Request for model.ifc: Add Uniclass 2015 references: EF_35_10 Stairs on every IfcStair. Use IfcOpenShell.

First a look at what the model holds.

```python
import ifcopenshell

model = ifcopenshell.open("model.ifc")
print(model.schema)
print("classifications:", [c.Name for c in model.by_type("IfcClassification")])
for ifc_class in ("IfcDoor", "IfcRoof", "IfcStair", "IfcWall", "IfcWindow"):
    print(ifc_class, len(model.by_type(ifc_class)))
```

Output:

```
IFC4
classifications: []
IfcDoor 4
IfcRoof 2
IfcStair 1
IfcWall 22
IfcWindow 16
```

```python
import ifcopenshell
import ifcopenshell.api.classification

model = ifcopenshell.open("model.ifc")

system = ifcopenshell.api.classification.add_classification(model, classification="Uniclass 2015")

codes = {
    "IfcStair": ("EF_35_10", "Stairs"),
}
for ifc_class, (code, name) in codes.items():
    products = model.by_type(ifc_class)
    ifcopenshell.api.classification.add_reference(
        model, products=products, classification=system, identification=code, name=name
    )
    print(code, len(products))

model.write("model_edited.ifc")
```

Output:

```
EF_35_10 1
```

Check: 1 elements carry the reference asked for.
